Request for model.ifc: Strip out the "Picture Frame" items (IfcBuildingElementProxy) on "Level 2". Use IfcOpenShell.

First a look at what the model holds.

```python
import ifcopenshell
import ifcopenshell.util.element

model = ifcopenshell.open("model.ifc")
print(model.schema)
storey = next(s for s in model.by_type("IfcBuildingStorey") if s.Name == "Level 2")
proxies = [e for e in ifcopenshell.util.element.get_decomposition(storey) if e.is_a("IfcBuildingElementProxy")]
seen = {}
for e in proxies:
    element_type = ifcopenshell.util.element.get_type(e)
    name = element_type.Name if element_type not in (None, e) else None
    seen[name] = seen.get(name, 0) + 1
for name, count in sorted(seen.items(), key=str):
    print(count, "x", name)
```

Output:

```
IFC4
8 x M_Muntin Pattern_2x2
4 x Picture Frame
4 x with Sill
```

```python
import ifcopenshell
import ifcopenshell.api.root
import ifcopenshell.util.element

model = ifcopenshell.open("model.ifc")

storey = next(s for s in model.by_type("IfcBuildingStorey") if s.Name == "Level 2")
proxies = [e for e in ifcopenshell.util.element.get_decomposition(storey) if e.is_a("IfcBuildingElementProxy")]
targets = [e for e in proxies if (t := ifcopenshell.util.element.get_type(e)) not in (None, e) and t.Name == "Picture Frame"]

for e in targets:
    ifcopenshell.api.root.remove_product(model, product=e)
print(len(targets), "removed")

model.write("model_edited.ifc")
```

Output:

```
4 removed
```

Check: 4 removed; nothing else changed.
